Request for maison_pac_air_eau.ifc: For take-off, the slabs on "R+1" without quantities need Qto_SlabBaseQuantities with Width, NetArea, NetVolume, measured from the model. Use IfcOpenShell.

First a look at what the model holds.

```python
import ifcopenshell
import ifcopenshell.util.element
import ifcopenshell.util.unit

model = ifcopenshell.open("maison_pac_air_eau.ifc")
print(model.schema)
for unit_type in ("LENGTHUNIT", "AREAUNIT", "VOLUMEUNIT"):
    print(unit_type, ifcopenshell.util.unit.calculate_unit_scale(model, unit_type))
storey = next(s for s in model.by_type("IfcBuildingStorey") if s.Name == "R+1")
slabs = [e for e in ifcopenshell.util.element.get_decomposition(storey) if e.is_a("IfcSlab")]
for e in sorted(slabs, key=lambda e: e.id()):
    print(e.id(), e.is_a(), e.Name, list(ifcopenshell.util.element.get_psets(e, qtos_only=True)), sep=" | ")
```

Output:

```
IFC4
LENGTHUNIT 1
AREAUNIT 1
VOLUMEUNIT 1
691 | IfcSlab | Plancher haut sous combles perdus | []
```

```python
import ifcopenshell
import ifcopenshell.api.pset
import ifcopenshell.geom
import ifcopenshell.util.element
import ifcopenshell.util.shape
import ifcopenshell.util.unit

model = ifcopenshell.open("maison_pac_air_eau.ifc")
unit_scale = ifcopenshell.util.unit.calculate_unit_scale(model)
area_scale = ifcopenshell.util.unit.calculate_unit_scale(model, "AREAUNIT")
volume_scale = ifcopenshell.util.unit.calculate_unit_scale(model, "VOLUMEUNIT")
settings = ifcopenshell.geom.settings()

storey = next(s for s in model.by_type("IfcBuildingStorey") if s.Name == "R+1")
slabs = [e for e in ifcopenshell.util.element.get_decomposition(storey) if e.is_a("IfcSlab")]

for e in sorted(slabs, key=lambda e: e.id()):
    if ifcopenshell.util.element.get_psets(e, qtos_only=True, should_inherit=False):
        continue
    # Geometry comes back in metres, in the element's own axes.
    shape = ifcopenshell.geom.create_shape(settings, e)
    values = {
        "Width": ifcopenshell.util.shape.get_z(shape.geometry) / unit_scale,
        "NetArea": ifcopenshell.util.shape.get_footprint_area(shape.geometry) / area_scale,
        "NetVolume": ifcopenshell.util.shape.get_volume(shape.geometry) / volume_scale,
    }
    qto = ifcopenshell.api.pset.add_qto(model, product=e, name="Qto_SlabBaseQuantities")
    ifcopenshell.api.pset.edit_qto(model, qto=qto, properties=values)
    print(e.id(), {k: round(v, 3) for k, v in values.items()})

model.write("maison_pac_air_eau-out.ifc")
```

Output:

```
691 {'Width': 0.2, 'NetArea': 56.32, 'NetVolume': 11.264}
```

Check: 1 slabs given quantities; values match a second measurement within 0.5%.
